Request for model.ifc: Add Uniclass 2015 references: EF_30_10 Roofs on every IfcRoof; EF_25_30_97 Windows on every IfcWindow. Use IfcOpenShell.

First a look at what the model holds.

```python
import ifcopenshell

model = ifcopenshell.open("model.ifc")
print(model.schema)
print("classifications:", [c.Name for c in model.by_type("IfcClassification")])
for ifc_class in ("IfcDoor", "IfcRoof", "IfcStair", "IfcWall", "IfcWindow"):
    print(ifc_class, len(model.by_type(ifc_class)))
```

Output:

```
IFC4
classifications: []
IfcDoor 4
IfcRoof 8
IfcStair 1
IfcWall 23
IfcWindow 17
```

```python
import ifcopenshell
import ifcopenshell.api.classification

model = ifcopenshell.open("model.ifc")

system = ifcopenshell.api.classification.add_classification(model, classification="Uniclass 2015")

codes = {
    "IfcRoof": ("EF_30_10", "Roofs"),
    "IfcWindow": ("EF_25_30_97", "Windows"),
}
for ifc_class, (code, name) in codes.items():
    products = model.by_type(ifc_class)
    ifcopenshell.api.classification.add_reference(
        model, products=products, classification=system, identification=code, name=name
    )
    print(code, len(products))

model.write("model-out.ifc")
```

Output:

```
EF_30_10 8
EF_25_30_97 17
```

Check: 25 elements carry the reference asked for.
